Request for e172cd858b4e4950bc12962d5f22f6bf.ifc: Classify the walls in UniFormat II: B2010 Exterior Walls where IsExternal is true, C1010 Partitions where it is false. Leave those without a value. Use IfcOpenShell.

First a look at what the model holds.

```python
import ifcopenshell
import ifcopenshell.util.element

model = ifcopenshell.open("e172cd858b4e4950bc12962d5f22f6bf.ifc")
print(model.schema)
print("classifications:", [c.Name for c in model.by_type("IfcClassification")])
values = [ifcopenshell.util.element.get_pset(e, "Pset_WallCommon", "IsExternal") for e in model.by_type("IfcWall")]
for value in (True, False, None):
    print("IsExternal", value, values.count(value))
```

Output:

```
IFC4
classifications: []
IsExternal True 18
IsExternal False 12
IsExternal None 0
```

```python
import ifcopenshell
import ifcopenshell.api.classification
import ifcopenshell.util.element

model = ifcopenshell.open("e172cd858b4e4950bc12962d5f22f6bf.ifc")

system = ifcopenshell.api.classification.add_classification(model, classification="UniFormat II")

walls = model.by_type("IfcWall")
external = {e: ifcopenshell.util.element.get_pset(e, "Pset_WallCommon", "IsExternal") for e in walls}
for flag, code, name in ((True, "B2010", "Exterior Walls"), (False, "C1010", "Partitions")):
    products = [e for e in walls if external[e] is flag]
    ifcopenshell.api.classification.add_reference(
        model, products=products, classification=system, identification=code, name=name
    )
    print(code, len(products))

model.write("e172cd858b4e4950bc12962d5f22f6bf-out.ifc")
```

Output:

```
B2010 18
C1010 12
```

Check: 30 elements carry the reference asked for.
